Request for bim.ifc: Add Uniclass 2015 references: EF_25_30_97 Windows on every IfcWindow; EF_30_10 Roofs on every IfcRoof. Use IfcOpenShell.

First a look at what the model holds.

```python
import ifcopenshell

model = ifcopenshell.open("bim.ifc")
print(model.schema)
print("classifications:", [c.Name for c in model.by_type("IfcClassification")])
for ifc_class in ("IfcDoor", "IfcRoof", "IfcStair", "IfcWall", "IfcWindow"):
    print(ifc_class, len(model.by_type(ifc_class)))
```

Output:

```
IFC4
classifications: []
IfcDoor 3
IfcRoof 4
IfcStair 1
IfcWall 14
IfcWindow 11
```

```python
import ifcopenshell
import ifcopenshell.api.classification

model = ifcopenshell.open("bim.ifc")

system = ifcopenshell.api.classification.add_classification(model, classification="Uniclass 2015")

codes = {
    "IfcWindow": ("EF_25_30_97", "Windows"),
    "IfcRoof": ("EF_30_10", "Roofs"),
}
for ifc_class, (code, name) in codes.items():
    products = model.by_type(ifc_class)
    ifcopenshell.api.classification.add_reference(
        model, products=products, classification=system, identification=code, name=name
    )
    print(code, len(products))

model.write("bim-out.ifc")
```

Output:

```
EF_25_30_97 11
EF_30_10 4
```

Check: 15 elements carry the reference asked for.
